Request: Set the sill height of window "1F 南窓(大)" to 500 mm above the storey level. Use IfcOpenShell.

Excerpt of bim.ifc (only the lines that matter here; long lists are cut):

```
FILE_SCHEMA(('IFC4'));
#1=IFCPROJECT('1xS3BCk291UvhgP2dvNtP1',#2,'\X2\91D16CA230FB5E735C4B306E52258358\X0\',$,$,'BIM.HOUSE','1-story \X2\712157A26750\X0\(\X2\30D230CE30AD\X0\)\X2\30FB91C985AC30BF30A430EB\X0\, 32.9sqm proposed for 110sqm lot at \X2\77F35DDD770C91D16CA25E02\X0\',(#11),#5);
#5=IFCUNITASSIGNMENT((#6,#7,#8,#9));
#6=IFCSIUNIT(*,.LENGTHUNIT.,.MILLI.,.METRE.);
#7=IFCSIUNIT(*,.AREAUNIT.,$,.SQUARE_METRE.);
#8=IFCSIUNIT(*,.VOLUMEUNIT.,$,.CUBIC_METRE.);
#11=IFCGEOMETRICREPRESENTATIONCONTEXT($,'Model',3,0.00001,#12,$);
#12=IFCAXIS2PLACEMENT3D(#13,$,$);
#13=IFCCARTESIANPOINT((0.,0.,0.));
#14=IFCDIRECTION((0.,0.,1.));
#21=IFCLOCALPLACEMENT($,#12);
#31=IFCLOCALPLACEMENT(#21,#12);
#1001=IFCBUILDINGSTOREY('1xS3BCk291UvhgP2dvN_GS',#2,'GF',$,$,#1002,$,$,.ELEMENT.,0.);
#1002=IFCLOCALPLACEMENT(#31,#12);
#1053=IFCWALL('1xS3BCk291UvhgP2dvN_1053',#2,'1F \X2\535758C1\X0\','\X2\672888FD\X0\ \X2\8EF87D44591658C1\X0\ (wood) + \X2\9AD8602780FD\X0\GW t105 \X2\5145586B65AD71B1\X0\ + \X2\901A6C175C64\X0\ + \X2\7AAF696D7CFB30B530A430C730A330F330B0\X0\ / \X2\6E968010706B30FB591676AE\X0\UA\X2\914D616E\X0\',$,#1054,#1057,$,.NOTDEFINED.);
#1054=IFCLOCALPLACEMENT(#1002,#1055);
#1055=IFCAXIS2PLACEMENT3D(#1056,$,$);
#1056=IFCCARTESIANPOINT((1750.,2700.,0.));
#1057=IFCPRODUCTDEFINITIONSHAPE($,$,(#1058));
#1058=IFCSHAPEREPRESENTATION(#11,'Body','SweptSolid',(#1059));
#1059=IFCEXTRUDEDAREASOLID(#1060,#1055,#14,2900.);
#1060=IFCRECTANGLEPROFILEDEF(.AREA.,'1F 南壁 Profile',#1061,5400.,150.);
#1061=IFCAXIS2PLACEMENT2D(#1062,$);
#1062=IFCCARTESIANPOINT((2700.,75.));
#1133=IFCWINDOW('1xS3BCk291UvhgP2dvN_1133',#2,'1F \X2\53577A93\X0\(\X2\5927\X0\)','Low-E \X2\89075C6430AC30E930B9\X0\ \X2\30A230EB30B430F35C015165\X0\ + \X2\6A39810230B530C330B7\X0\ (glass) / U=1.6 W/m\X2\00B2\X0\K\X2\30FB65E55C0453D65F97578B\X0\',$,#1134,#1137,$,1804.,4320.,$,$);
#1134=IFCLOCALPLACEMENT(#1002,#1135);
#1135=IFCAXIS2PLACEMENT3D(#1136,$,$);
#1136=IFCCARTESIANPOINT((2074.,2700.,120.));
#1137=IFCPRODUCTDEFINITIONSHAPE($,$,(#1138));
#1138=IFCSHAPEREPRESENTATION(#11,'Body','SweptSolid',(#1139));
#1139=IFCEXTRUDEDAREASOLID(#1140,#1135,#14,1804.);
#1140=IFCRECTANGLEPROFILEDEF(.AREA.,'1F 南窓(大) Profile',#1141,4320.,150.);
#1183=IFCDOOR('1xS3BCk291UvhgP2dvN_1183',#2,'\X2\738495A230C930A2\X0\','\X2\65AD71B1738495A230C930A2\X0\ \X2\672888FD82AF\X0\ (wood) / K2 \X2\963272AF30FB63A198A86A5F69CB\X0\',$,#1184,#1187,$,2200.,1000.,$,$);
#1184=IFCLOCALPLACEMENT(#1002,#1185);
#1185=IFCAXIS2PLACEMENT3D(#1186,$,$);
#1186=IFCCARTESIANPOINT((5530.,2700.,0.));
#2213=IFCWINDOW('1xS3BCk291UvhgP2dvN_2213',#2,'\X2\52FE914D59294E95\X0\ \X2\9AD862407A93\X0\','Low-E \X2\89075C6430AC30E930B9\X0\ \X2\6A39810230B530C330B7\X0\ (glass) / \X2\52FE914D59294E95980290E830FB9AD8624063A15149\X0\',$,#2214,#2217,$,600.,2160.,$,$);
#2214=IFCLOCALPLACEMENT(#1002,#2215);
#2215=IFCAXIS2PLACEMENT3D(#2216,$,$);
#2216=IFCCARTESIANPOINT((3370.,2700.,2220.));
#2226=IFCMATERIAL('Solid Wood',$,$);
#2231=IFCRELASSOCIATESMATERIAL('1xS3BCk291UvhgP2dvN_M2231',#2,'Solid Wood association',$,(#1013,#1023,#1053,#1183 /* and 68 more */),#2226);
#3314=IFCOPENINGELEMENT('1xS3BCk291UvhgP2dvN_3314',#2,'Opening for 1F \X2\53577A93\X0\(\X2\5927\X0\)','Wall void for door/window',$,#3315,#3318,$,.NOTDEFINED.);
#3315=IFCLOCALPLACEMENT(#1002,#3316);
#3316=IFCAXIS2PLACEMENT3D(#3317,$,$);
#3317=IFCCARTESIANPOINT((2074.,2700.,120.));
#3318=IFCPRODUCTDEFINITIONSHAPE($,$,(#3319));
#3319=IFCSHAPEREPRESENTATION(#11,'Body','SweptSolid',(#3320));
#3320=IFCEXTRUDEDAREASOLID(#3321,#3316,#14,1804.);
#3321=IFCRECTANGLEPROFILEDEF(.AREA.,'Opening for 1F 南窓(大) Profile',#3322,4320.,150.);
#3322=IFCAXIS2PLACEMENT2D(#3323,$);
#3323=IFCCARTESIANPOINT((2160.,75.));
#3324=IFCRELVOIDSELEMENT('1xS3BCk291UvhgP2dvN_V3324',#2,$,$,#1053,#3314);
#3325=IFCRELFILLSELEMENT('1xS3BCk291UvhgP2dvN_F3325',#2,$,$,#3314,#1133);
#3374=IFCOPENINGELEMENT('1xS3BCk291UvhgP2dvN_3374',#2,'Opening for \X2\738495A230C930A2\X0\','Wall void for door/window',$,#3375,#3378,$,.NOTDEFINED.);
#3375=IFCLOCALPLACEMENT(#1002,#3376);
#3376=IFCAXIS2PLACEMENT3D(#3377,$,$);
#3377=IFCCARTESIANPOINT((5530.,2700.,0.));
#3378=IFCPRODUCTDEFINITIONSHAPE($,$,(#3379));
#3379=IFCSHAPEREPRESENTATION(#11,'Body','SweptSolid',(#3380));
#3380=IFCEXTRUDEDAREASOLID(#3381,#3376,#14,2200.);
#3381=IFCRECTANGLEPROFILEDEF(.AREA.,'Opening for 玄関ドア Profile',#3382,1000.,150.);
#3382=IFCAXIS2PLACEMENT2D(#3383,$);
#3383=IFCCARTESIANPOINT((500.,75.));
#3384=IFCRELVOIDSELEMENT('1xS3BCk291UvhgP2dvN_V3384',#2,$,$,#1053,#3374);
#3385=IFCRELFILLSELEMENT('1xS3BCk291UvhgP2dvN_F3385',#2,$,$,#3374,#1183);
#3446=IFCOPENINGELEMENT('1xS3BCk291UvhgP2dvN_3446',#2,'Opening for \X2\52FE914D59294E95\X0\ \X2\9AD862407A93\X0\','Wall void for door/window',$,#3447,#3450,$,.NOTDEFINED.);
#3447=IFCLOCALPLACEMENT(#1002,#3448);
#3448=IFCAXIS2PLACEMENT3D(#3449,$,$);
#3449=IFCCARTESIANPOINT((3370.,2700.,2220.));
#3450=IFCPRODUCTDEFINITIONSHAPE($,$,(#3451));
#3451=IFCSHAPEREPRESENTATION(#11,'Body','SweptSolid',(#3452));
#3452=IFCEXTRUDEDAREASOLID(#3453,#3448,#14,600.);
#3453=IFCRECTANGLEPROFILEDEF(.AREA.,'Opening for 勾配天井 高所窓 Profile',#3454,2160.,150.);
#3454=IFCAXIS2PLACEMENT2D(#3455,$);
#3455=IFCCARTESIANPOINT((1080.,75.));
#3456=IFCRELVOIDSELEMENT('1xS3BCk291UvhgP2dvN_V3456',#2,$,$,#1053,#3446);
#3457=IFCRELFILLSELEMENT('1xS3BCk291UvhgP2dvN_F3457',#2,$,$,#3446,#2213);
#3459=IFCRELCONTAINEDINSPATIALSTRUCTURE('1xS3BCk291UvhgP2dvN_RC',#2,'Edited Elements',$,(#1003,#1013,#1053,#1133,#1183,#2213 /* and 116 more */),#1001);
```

```python
import numpy as np
import ifcopenshell
import ifcopenshell.api.geometry
import ifcopenshell.geom
import ifcopenshell.util.element
import ifcopenshell.util.placement
import ifcopenshell.util.shape
import ifcopenshell.util.unit

model = ifcopenshell.open("bim.ifc")
unit_scale = ifcopenshell.util.unit.calculate_unit_scale(model)

window = model.by_guid("1xS3BCk291UvhgP2dvN_1133")
opening = window.FillsVoids[0].RelatingOpeningElement
storey = ifcopenshell.util.element.get_container(window, ifc_class="IfcBuildingStorey")
level = ifcopenshell.util.placement.get_local_placement(storey.ObjectPlacement)[2, 3]

# The opening's origin need not be at the sill, so measure its lowest point.
shape = ifcopenshell.geom.create_shape(ifcopenshell.geom.settings(), opening)
bottom = ifcopenshell.util.shape.get_shape_bottom_elevation(shape, shape.geometry) / unit_scale
dz = level + 500.0 - bottom

shift = np.array([0.0, 0.0, dz])
# The window is not placed relative to its opening, so move both.
for product in (opening, window):
    matrix = ifcopenshell.util.placement.get_local_placement(product.ObjectPlacement)
    matrix[:3, 3] += shift
    ifcopenshell.api.geometry.edit_object_placement(model, product=product, matrix=matrix, is_si=False)

print(f"moved by {dz * unit_scale:+.3f} m")

model.write("bim-out.ifc")
```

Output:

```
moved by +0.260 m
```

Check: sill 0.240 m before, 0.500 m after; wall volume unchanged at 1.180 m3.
